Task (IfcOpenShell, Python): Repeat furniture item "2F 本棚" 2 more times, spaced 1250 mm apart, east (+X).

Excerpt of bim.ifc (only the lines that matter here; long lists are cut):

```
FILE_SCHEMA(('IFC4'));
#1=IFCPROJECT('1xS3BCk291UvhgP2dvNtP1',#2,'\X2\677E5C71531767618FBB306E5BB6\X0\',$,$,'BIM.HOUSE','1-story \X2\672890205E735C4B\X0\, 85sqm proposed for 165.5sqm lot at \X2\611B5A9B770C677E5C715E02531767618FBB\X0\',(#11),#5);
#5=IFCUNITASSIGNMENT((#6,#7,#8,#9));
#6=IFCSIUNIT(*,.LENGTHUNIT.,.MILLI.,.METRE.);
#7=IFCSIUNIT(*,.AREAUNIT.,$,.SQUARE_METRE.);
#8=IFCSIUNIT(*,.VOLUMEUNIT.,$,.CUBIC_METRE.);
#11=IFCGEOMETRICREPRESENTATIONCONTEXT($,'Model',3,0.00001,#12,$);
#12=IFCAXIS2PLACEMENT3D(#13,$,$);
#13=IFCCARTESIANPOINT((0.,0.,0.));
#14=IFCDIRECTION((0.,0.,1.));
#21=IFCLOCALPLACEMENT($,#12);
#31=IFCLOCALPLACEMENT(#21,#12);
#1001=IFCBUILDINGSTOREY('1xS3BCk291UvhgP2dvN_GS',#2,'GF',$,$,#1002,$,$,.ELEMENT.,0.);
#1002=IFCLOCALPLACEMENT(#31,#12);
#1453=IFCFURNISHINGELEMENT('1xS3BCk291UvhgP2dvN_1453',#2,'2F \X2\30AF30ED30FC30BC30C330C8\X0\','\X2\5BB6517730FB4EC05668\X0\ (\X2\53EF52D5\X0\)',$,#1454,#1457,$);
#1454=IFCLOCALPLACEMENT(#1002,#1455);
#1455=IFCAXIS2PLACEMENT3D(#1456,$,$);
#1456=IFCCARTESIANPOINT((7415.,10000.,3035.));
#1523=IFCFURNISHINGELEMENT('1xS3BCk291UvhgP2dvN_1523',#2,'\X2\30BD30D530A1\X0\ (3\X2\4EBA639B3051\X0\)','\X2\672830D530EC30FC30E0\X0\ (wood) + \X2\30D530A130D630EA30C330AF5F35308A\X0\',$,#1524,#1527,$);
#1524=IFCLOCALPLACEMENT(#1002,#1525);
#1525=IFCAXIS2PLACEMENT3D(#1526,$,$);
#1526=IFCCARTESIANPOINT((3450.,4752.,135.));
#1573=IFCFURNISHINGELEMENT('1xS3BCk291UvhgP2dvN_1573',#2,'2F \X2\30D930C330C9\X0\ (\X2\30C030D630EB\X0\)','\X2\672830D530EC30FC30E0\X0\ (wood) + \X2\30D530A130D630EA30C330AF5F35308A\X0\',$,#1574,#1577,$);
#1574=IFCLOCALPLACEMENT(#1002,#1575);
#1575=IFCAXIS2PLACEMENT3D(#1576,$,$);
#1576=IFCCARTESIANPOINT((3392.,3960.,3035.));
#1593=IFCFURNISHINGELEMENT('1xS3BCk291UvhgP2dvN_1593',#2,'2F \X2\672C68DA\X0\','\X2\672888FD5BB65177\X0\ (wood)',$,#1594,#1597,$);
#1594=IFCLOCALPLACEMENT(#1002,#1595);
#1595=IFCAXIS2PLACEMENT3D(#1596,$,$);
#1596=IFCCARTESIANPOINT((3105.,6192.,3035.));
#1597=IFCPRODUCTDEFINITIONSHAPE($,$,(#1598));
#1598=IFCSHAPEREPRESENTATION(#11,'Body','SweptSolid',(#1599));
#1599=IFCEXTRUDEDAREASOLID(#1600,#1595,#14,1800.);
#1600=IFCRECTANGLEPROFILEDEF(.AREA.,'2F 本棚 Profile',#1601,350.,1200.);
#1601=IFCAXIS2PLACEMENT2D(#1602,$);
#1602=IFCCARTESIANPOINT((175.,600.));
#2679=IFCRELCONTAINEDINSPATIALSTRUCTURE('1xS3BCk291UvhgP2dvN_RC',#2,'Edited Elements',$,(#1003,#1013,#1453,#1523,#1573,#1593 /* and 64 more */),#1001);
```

```python
import numpy as np
import ifcopenshell
import ifcopenshell.api.geometry
import ifcopenshell.api.root
import ifcopenshell.util.element
import ifcopenshell.util.placement
import ifcopenshell.util.unit

model = ifcopenshell.open("bim.ifc")
unit_scale = ifcopenshell.util.unit.calculate_unit_scale(model)


def reuse_history(source, copy):
    """copy_class also copies each property set's owner history, people and application; keep the originals."""
    for rel in copy.IsDefinedBy:
        if rel.is_a("IfcRelDefinesByProperties") and (history := rel.RelatingPropertyDefinition.OwnerHistory):
            rel.RelatingPropertyDefinition.OwnerHistory = source.OwnerHistory
            ifcopenshell.util.element.remove_deep2(model, history)


source = model.by_guid("1xS3BCk291UvhgP2dvN_1593")
base = ifcopenshell.util.placement.get_local_placement(source.ObjectPlacement)
step = np.array([1.0, 0.0, 0.0]) * 1.25 / unit_scale

for i in range(1, 3):
    copy = ifcopenshell.api.root.copy_class(model, product=source)
    copy.Representation = ifcopenshell.util.element.copy_deep(
        model, source.Representation, exclude=["IfcGeometricRepresentationContext", "IfcRepresentationMap"]
    )
    reuse_history(source, copy)
    matrix = base.copy()
    matrix[:3, 3] += i * step
    print("added at", matrix[:3, 3].round(3) + 0.0)
    ifcopenshell.api.geometry.edit_object_placement(model, product=copy, matrix=matrix, is_si=False)

model.write("bim-out.ifc")
```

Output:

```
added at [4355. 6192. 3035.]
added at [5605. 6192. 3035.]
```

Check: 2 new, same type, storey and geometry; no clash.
